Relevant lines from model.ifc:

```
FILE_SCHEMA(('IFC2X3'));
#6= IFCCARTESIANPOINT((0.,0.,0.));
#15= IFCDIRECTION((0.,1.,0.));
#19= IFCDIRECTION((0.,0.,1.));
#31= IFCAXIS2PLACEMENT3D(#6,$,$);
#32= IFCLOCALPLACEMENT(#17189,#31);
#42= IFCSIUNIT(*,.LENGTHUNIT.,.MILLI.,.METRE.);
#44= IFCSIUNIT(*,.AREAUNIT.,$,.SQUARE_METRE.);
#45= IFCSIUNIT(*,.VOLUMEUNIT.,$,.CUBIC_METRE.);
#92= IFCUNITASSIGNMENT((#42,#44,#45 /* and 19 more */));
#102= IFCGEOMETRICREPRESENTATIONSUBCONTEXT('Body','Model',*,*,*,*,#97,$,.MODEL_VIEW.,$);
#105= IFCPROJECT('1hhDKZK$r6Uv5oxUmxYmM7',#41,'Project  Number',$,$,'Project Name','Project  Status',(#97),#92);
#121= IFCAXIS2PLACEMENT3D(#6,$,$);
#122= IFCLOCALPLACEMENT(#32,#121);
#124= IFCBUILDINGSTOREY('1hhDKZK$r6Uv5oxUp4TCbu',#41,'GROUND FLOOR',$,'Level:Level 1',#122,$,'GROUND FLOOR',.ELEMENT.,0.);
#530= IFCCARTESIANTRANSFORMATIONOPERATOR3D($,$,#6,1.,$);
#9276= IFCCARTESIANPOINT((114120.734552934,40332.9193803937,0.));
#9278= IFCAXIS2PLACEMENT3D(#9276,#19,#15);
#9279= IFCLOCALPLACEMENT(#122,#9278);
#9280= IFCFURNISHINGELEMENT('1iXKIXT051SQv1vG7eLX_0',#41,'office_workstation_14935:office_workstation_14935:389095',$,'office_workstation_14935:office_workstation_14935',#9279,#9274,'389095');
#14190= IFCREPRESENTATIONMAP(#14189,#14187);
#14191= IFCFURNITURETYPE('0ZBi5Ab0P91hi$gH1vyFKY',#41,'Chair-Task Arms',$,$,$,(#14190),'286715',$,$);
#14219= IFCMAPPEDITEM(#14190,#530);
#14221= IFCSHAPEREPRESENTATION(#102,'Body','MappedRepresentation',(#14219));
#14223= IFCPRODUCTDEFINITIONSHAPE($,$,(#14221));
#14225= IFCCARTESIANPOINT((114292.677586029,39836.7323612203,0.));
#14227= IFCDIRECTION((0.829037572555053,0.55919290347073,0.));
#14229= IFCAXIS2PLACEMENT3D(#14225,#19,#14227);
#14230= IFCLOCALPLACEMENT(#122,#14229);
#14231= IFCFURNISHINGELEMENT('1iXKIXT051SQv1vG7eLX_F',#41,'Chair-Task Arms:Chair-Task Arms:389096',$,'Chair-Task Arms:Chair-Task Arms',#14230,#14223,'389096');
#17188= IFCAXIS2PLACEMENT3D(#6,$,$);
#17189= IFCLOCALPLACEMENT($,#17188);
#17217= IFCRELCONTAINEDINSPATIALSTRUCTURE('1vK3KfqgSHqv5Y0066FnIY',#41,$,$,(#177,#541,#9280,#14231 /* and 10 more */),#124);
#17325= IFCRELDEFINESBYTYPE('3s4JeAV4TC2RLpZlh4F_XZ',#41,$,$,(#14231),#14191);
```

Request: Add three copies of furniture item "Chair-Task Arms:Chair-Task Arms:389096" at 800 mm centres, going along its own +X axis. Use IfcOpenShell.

```python
import ifcopenshell
import ifcopenshell.api.geometry
import ifcopenshell.api.root
import ifcopenshell.util.element
import ifcopenshell.util.placement
import ifcopenshell.util.unit

model = ifcopenshell.open("model.ifc")
unit_scale = ifcopenshell.util.unit.calculate_unit_scale(model)


def reuse_history(source, copy):
    """copy_class also copies each property set's owner history, people and application; keep the originals."""
    for rel in copy.IsDefinedBy:
        if rel.is_a("IfcRelDefinesByProperties") and (history := rel.RelatingPropertyDefinition.OwnerHistory):
            rel.RelatingPropertyDefinition.OwnerHistory = source.OwnerHistory
            ifcopenshell.util.element.remove_deep2(model, history)


source = model.by_guid("1iXKIXT051SQv1vG7eLX_F")
base = ifcopenshell.util.placement.get_local_placement(source.ObjectPlacement)
step = base[:3, 0] * 0.8 / unit_scale

for i in range(1, 4):
    copy = ifcopenshell.api.root.copy_class(model, product=source)
    copy.Representation = ifcopenshell.util.element.copy_deep(
        model, source.Representation, exclude=["IfcGeometricRepresentationContext", "IfcRepresentationMap"]
    )
    copy.Name = "Chair-Task Arms:Chair-Task Arms"
    copy.Tag = None
    reuse_history(source, copy)
    matrix = base.copy()
    matrix[:3, 3] += i * step
    print("added at", matrix[:3, 3].round(3) + 0.0)
    ifcopenshell.api.geometry.edit_object_placement(model, product=copy, matrix=matrix, is_si=False)

model.write("model_edited.ifc")
```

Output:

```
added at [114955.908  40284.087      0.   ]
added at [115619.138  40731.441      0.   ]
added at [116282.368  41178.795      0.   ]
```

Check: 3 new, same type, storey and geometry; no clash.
